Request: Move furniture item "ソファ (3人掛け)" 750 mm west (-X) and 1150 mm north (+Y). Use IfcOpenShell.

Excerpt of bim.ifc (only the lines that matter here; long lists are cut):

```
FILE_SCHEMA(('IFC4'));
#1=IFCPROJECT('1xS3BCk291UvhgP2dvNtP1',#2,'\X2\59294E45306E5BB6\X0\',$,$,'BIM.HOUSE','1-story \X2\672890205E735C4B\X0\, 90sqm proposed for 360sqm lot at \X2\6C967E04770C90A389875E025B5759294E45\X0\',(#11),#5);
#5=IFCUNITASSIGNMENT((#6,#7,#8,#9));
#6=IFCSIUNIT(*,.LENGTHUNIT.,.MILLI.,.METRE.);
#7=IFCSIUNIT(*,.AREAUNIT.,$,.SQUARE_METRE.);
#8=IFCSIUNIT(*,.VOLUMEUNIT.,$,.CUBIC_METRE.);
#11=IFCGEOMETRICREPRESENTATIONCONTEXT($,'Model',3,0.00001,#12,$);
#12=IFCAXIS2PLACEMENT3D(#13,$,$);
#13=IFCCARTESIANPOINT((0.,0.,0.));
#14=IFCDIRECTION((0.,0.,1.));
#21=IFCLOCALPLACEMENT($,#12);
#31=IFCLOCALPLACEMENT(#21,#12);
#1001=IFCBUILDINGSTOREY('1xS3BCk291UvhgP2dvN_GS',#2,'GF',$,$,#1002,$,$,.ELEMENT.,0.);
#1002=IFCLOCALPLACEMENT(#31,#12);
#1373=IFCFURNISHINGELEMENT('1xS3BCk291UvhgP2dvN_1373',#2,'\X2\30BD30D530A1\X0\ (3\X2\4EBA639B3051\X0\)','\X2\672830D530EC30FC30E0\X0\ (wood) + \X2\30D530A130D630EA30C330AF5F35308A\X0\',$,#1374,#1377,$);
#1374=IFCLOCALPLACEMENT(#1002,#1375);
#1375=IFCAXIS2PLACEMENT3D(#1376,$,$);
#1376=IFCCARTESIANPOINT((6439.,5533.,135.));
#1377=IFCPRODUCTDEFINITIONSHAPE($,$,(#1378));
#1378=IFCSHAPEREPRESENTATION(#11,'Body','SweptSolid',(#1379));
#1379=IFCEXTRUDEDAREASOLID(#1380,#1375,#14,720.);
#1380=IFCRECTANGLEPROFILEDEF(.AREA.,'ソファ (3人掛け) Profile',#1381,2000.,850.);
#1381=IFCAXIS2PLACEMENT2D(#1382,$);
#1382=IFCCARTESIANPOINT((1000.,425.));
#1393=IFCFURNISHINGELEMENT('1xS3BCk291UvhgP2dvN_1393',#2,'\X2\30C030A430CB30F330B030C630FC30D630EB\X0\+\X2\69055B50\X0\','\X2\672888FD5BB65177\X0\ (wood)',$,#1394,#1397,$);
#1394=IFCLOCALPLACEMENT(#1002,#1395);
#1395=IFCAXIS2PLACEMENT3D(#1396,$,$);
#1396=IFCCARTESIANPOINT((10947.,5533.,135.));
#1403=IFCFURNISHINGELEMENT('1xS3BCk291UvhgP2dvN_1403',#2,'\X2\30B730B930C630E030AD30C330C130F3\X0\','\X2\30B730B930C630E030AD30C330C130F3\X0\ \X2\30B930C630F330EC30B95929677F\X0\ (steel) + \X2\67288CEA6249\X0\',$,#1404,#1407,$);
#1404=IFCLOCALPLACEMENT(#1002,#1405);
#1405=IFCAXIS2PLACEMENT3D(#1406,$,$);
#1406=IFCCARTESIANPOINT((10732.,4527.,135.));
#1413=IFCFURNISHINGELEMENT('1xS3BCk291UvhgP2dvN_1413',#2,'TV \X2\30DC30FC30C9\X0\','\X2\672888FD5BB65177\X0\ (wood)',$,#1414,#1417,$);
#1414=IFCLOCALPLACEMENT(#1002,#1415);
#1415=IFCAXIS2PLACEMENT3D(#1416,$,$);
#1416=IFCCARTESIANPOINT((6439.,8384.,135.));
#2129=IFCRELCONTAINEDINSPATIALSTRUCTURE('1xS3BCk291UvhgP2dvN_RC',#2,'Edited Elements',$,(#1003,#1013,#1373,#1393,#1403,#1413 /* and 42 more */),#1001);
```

```python
import ifcopenshell
import ifcopenshell.api.geometry
import ifcopenshell.util.placement

model = ifcopenshell.open("bim.ifc")

item = model.by_guid("1xS3BCk291UvhgP2dvN_1373")
matrix = ifcopenshell.util.placement.get_local_placement(item.ObjectPlacement)
matrix[0, 3] -= 750.0
matrix[1, 3] += 1150.0
ifcopenshell.api.geometry.edit_object_placement(model, product=item, matrix=matrix, is_si=False)

print(ifcopenshell.util.placement.get_local_placement(item.ObjectPlacement).round(3) + 0.0)

model.write("bim_edited.ifc")
```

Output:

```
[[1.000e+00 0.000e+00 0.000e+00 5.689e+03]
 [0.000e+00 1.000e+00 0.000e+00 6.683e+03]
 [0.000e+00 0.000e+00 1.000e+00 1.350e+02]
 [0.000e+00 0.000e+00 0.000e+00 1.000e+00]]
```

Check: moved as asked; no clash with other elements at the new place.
